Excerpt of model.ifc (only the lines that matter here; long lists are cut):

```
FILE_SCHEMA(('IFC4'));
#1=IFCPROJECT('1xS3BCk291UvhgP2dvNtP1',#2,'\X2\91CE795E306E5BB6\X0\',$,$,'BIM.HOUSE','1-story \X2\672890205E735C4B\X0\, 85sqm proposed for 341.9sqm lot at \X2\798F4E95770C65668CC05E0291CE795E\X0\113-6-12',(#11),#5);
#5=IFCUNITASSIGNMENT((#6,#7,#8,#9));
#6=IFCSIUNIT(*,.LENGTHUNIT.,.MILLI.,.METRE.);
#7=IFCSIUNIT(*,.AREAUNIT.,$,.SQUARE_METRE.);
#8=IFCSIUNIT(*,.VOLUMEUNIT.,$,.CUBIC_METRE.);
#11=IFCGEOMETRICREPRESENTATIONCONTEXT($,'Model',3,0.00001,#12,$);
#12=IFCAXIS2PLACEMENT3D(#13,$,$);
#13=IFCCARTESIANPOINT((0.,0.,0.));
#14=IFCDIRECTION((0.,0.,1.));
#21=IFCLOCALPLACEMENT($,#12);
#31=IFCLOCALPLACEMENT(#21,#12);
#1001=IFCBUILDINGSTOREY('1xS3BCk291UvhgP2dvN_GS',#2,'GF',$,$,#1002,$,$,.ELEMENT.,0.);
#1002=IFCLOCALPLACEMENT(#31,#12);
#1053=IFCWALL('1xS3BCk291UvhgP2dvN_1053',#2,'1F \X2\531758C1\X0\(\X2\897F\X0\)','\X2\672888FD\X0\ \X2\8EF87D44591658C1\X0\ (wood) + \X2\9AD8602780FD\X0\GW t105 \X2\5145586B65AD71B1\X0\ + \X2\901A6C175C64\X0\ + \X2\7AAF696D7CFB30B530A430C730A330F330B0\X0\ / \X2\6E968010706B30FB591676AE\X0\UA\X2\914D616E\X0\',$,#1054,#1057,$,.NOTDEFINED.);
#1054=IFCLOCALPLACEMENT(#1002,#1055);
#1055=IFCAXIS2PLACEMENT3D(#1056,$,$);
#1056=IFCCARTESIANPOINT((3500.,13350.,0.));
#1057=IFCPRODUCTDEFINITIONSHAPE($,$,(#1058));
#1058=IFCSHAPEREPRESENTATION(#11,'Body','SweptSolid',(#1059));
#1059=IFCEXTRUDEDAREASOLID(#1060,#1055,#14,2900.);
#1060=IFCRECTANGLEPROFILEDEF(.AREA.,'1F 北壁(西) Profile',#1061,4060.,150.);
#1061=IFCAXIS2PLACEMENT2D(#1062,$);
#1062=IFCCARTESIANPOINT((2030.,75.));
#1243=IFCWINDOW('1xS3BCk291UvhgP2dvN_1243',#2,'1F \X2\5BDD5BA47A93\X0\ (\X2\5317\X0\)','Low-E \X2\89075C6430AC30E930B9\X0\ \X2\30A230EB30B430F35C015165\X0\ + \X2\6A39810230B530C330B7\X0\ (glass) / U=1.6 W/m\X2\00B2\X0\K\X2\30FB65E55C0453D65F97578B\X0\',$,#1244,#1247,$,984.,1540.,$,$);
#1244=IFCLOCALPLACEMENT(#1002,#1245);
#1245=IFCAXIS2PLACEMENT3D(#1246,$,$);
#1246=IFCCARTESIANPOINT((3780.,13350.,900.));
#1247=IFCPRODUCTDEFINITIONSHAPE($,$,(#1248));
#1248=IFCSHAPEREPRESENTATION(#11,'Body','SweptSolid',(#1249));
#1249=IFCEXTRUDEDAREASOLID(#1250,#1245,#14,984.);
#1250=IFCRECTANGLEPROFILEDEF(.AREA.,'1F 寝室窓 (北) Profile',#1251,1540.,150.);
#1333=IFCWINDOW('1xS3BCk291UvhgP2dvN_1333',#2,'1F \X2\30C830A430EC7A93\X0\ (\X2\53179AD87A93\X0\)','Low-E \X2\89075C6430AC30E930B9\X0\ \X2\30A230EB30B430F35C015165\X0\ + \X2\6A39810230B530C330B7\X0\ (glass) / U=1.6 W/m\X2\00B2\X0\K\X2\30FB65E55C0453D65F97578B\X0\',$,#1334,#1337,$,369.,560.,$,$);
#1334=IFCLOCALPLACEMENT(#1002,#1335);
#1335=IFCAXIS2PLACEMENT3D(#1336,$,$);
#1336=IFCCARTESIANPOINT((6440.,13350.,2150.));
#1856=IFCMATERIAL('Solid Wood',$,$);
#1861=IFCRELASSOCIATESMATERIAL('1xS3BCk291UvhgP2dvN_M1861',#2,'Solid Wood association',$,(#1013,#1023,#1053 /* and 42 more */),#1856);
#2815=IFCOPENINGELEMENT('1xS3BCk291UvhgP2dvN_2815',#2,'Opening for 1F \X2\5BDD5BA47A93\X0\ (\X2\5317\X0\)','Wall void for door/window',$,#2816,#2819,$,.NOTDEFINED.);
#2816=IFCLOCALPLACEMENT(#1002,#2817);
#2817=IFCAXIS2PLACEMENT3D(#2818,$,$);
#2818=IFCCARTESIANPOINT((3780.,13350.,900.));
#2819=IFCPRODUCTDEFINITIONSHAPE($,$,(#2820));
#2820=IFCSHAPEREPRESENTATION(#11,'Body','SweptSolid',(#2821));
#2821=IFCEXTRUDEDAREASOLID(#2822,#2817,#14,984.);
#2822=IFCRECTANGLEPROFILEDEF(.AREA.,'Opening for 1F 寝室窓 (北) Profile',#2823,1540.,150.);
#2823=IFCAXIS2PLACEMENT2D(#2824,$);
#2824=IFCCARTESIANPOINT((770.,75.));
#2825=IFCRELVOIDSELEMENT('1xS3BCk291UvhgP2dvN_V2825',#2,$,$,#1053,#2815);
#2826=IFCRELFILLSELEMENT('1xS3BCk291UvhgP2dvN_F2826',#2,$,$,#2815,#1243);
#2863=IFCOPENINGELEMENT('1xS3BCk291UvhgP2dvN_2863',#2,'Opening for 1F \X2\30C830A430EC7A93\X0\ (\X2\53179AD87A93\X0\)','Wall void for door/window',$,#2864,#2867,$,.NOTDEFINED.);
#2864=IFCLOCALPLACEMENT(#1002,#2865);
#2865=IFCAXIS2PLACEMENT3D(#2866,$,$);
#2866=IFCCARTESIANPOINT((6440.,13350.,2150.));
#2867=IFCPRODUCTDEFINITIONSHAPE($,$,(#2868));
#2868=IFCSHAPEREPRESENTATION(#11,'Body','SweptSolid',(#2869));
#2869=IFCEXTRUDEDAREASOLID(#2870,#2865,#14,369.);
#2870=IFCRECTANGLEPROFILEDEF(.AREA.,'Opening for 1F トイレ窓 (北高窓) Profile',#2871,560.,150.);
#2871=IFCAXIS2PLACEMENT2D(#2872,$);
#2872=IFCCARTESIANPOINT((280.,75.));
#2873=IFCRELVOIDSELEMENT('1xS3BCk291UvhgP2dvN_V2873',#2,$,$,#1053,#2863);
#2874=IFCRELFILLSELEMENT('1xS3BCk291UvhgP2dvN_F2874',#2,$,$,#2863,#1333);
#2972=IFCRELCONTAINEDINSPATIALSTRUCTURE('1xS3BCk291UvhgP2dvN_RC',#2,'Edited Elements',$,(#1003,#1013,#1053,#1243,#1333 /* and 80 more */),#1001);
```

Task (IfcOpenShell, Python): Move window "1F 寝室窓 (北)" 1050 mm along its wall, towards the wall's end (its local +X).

```python
import ifcopenshell
import ifcopenshell.api.geometry
import ifcopenshell.util.placement

model = ifcopenshell.open("model.ifc")

window = model.by_guid("1xS3BCk291UvhgP2dvN_1243")
opening = window.FillsVoids[0].RelatingOpeningElement
wall = opening.VoidsElements[0].RelatingBuildingElement

wall_matrix = ifcopenshell.util.placement.get_local_placement(wall.ObjectPlacement)
shift = wall_matrix[:3, 0] * 1050.0
before = ifcopenshell.util.placement.get_local_placement(window.ObjectPlacement)[:3, 3].copy()

# The window is not placed relative to its opening, so move both.
for product in (opening, window):
    matrix = ifcopenshell.util.placement.get_local_placement(product.ObjectPlacement)
    matrix[:3, 3] += shift
    ifcopenshell.api.geometry.edit_object_placement(model, product=product, matrix=matrix, is_si=False)

after = ifcopenshell.util.placement.get_local_placement(window.ObjectPlacement)[:3, 3]
print("window moved by", (after - before).round(3) + 0.0)

model.write("model_updated.ifc")
```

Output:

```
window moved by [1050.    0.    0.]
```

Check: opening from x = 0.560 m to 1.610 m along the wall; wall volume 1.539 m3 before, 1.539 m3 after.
